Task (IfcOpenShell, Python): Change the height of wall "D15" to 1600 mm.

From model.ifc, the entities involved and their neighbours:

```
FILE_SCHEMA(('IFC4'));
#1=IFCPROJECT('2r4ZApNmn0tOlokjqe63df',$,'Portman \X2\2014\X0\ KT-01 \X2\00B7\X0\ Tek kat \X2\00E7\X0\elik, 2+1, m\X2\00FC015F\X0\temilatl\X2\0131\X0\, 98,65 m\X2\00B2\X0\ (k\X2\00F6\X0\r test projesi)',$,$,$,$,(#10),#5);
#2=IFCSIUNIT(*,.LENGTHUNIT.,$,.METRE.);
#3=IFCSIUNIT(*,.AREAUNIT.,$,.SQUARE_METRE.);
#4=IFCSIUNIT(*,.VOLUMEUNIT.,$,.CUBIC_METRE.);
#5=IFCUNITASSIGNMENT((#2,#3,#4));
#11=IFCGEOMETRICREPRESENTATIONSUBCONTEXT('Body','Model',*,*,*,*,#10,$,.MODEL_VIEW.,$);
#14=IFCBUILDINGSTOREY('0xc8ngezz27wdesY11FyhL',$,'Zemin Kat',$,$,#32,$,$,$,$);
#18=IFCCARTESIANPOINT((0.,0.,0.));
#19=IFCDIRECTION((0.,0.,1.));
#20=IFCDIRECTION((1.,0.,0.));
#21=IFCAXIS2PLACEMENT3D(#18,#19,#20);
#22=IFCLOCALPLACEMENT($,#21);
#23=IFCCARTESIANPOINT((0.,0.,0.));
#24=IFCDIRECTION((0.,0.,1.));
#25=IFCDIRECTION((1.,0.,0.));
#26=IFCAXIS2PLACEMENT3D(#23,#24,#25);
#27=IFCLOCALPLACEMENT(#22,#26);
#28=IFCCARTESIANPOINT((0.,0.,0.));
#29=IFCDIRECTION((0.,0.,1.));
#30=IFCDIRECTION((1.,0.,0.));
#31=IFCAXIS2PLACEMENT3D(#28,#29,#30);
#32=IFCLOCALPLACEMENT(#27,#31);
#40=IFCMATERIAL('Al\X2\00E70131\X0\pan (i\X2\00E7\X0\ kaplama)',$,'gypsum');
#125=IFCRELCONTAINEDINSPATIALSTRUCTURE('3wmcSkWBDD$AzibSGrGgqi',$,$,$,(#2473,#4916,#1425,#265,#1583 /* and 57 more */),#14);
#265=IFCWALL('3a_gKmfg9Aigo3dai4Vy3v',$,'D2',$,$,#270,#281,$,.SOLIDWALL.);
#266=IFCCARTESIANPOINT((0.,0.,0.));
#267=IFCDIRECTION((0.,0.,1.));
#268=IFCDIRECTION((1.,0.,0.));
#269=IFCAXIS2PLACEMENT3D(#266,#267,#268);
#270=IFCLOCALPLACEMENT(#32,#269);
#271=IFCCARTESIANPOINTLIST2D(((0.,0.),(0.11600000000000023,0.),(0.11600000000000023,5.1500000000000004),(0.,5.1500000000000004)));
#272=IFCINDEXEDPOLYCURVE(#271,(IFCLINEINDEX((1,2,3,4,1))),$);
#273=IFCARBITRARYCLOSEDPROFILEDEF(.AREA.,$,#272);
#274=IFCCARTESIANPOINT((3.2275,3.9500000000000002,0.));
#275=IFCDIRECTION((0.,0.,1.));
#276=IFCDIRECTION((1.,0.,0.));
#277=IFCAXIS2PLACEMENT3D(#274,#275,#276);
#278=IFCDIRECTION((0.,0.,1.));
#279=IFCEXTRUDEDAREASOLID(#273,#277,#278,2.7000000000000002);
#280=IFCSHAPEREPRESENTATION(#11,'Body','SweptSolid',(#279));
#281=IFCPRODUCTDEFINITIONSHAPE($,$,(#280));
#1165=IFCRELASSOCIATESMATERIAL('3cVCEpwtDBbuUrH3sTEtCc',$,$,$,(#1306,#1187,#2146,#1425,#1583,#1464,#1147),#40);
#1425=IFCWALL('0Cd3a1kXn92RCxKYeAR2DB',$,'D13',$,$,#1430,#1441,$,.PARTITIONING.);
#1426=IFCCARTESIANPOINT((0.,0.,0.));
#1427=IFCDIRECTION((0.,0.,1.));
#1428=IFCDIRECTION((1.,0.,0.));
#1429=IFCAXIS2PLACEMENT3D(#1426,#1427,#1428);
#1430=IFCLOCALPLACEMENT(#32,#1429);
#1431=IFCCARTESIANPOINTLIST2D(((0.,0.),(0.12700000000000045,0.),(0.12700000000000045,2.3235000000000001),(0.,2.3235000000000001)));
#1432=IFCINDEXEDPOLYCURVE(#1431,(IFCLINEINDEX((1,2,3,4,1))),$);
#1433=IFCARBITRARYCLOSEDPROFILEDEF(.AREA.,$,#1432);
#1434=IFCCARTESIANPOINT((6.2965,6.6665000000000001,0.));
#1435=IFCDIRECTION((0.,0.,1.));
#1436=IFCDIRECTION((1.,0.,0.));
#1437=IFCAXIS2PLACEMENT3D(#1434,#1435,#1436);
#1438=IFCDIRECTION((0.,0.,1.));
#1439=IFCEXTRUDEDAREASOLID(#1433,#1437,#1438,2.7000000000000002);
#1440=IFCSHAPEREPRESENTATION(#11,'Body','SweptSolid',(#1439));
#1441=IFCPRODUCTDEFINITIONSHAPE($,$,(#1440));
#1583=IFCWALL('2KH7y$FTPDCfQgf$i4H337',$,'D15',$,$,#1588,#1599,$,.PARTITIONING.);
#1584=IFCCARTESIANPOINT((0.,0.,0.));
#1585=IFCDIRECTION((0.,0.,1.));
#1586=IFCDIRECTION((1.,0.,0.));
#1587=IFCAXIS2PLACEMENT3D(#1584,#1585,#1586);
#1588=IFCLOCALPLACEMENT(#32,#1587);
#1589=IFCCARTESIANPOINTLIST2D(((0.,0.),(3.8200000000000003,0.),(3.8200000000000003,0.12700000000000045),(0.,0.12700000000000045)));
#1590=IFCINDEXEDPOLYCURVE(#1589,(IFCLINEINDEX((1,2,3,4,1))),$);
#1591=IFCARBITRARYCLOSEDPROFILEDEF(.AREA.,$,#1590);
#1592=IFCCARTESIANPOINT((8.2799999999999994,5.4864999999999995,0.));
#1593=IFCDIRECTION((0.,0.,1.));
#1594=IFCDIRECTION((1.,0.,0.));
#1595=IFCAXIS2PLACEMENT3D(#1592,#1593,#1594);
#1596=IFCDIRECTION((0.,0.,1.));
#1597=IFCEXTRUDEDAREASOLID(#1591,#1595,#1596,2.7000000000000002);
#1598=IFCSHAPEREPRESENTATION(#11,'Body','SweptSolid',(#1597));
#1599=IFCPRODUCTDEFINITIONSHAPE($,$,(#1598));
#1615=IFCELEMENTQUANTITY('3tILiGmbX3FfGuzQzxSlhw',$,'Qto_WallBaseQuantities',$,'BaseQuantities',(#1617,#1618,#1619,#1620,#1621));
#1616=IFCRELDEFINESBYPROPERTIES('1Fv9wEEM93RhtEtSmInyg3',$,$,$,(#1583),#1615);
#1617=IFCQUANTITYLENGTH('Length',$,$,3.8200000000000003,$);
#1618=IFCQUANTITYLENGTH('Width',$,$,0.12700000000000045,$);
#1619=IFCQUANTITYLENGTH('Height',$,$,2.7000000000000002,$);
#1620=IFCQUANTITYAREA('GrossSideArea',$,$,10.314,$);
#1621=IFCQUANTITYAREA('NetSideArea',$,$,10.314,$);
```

```python
import ifcopenshell
import ifcopenshell.api.pset
import ifcopenshell.geom
import ifcopenshell.util.element
import ifcopenshell.util.representation
import ifcopenshell.util.shape
import ifcopenshell.util.unit

model = ifcopenshell.open("model.ifc")
unit_scale = ifcopenshell.util.unit.calculate_unit_scale(model)
area_scale = ifcopenshell.util.unit.calculate_unit_scale(model, "AREAUNIT")
settings = ifcopenshell.geom.settings()


def volume(element):
    """Net volume in cubic metres, openings subtracted."""
    shape = ifcopenshell.geom.create_shape(settings, element)
    return ifcopenshell.util.shape.get_volume(shape.geometry)


wall = model.by_guid("2KH7y$FTPDCfQgf$i4H337")
before = volume(wall)

body = ifcopenshell.util.representation.get_representation(wall, "Model", "Body")
solid = body.Items[0]
old_height = solid.Depth
solid.Depth = 1.6 / unit_scale
after = volume(wall)
thickness = 0.127  # wall thickness in metres

# Update the stored height, areas and volumes.
qto = model.by_id(ifcopenshell.util.element.get_pset(wall, "Qto_WallBaseQuantities", should_inherit=False)["id"])
ifcopenshell.api.pset.edit_qto(model, qto=qto, properties={
    "Height": solid.Depth,
    "GrossSideArea": ifcopenshell.util.element.get_pset(wall, "Qto_WallBaseQuantities", "GrossSideArea") * solid.Depth / old_height,
    "NetSideArea": after / thickness / area_scale,
})

print(f"height {old_height:g} -> {solid.Depth:g}, volume {before:.3f} -> {after:.3f} m3")

model.write("model-out.ifc")
```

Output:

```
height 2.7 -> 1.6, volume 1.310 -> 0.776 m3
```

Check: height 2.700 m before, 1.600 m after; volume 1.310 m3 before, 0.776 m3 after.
